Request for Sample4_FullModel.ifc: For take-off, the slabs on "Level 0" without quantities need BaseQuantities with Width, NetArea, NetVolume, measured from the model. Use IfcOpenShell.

First a look at what the model holds.

```python
import ifcopenshell
import ifcopenshell.util.element
import ifcopenshell.util.unit

model = ifcopenshell.open("Sample4_FullModel.ifc")
print(model.schema)
for unit_type in ("LENGTHUNIT", "AREAUNIT", "VOLUMEUNIT"):
    print(unit_type, ifcopenshell.util.unit.calculate_unit_scale(model, unit_type))
storey = next(s for s in model.by_type("IfcBuildingStorey") if s.Name == "Level 0")
slabs = [e for e in ifcopenshell.util.element.get_decomposition(storey) if e.is_a("IfcSlab")]
for e in sorted(slabs, key=lambda e: e.id()):
    print(e.id(), e.is_a(), e.Name, list(ifcopenshell.util.element.get_psets(e, qtos_only=True)), sep=" | ")
```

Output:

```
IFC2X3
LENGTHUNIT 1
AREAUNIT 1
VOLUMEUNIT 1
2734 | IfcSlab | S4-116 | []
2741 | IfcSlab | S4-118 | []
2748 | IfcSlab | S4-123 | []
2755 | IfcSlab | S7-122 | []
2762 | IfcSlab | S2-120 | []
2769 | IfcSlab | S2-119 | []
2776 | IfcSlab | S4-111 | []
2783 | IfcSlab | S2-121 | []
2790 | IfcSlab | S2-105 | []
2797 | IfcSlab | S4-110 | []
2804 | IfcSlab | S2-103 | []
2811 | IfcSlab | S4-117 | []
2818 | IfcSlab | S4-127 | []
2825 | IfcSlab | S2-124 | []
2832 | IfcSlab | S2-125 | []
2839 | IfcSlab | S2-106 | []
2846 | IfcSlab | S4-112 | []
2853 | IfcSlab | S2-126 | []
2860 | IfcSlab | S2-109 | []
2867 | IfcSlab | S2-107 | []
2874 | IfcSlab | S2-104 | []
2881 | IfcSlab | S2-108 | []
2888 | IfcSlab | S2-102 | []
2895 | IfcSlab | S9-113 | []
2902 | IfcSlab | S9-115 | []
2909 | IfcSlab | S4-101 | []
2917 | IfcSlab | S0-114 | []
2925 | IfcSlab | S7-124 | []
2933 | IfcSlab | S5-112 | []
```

```python
import ifcopenshell
import ifcopenshell.api.pset
import ifcopenshell.geom
import ifcopenshell.util.element
import ifcopenshell.util.shape
import ifcopenshell.util.unit

model = ifcopenshell.open("Sample4_FullModel.ifc")
unit_scale = ifcopenshell.util.unit.calculate_unit_scale(model)
area_scale = ifcopenshell.util.unit.calculate_unit_scale(model, "AREAUNIT")
volume_scale = ifcopenshell.util.unit.calculate_unit_scale(model, "VOLUMEUNIT")
settings = ifcopenshell.geom.settings()

storey = next(s for s in model.by_type("IfcBuildingStorey") if s.Name == "Level 0")
slabs = [e for e in ifcopenshell.util.element.get_decomposition(storey) if e.is_a("IfcSlab")]

for e in sorted(slabs, key=lambda e: e.id()):
    if ifcopenshell.util.element.get_psets(e, qtos_only=True, should_inherit=False):
        continue
    # Geometry comes back in metres, in the element's own axes.
    shape = ifcopenshell.geom.create_shape(settings, e)
    values = {
        "Width": ifcopenshell.util.shape.get_z(shape.geometry) / unit_scale,
        "NetArea": ifcopenshell.util.shape.get_footprint_area(shape.geometry) / area_scale,
        "NetVolume": ifcopenshell.util.shape.get_volume(shape.geometry) / volume_scale,
    }
    qto = ifcopenshell.api.pset.add_qto(model, product=e, name="BaseQuantities")
    ifcopenshell.api.pset.edit_qto(model, qto=qto, properties=values)
    print(e.id(), {k: round(v, 3) for k, v in values.items()})

model.write("Sample4_FullModel-out.ifc")
```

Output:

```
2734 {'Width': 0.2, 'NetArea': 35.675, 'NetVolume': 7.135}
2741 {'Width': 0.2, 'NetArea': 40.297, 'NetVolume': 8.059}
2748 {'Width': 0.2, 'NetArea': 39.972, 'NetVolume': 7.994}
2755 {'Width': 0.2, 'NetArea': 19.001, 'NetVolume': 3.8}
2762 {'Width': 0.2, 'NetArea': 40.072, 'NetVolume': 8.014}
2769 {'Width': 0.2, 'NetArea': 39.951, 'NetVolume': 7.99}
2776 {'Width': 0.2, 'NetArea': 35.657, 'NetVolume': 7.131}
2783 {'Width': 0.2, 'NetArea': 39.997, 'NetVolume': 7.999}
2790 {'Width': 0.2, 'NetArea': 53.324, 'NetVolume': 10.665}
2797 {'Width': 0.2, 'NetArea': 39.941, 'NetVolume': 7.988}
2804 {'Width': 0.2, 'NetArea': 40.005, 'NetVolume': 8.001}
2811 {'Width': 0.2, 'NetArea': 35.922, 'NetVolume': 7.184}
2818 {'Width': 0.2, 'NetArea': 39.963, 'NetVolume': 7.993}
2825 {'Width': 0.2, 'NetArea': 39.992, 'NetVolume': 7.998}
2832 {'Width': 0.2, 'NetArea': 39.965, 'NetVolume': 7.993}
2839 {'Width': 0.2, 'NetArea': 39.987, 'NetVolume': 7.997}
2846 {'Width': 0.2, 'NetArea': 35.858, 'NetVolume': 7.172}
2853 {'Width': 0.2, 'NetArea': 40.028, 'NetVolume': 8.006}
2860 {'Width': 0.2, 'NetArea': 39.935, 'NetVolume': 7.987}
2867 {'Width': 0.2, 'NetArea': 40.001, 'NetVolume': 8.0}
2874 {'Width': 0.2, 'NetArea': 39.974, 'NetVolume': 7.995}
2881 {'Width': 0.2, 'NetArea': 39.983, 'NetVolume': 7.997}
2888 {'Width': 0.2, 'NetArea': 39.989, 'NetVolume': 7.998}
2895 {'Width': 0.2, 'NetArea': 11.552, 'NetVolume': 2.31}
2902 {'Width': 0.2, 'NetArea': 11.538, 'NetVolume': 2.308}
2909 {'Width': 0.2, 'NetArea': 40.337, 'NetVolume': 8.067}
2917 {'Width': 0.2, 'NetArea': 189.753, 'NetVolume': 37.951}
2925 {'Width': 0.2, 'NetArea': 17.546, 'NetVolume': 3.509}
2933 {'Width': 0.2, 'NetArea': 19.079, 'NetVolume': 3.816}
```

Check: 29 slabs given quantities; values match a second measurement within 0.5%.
